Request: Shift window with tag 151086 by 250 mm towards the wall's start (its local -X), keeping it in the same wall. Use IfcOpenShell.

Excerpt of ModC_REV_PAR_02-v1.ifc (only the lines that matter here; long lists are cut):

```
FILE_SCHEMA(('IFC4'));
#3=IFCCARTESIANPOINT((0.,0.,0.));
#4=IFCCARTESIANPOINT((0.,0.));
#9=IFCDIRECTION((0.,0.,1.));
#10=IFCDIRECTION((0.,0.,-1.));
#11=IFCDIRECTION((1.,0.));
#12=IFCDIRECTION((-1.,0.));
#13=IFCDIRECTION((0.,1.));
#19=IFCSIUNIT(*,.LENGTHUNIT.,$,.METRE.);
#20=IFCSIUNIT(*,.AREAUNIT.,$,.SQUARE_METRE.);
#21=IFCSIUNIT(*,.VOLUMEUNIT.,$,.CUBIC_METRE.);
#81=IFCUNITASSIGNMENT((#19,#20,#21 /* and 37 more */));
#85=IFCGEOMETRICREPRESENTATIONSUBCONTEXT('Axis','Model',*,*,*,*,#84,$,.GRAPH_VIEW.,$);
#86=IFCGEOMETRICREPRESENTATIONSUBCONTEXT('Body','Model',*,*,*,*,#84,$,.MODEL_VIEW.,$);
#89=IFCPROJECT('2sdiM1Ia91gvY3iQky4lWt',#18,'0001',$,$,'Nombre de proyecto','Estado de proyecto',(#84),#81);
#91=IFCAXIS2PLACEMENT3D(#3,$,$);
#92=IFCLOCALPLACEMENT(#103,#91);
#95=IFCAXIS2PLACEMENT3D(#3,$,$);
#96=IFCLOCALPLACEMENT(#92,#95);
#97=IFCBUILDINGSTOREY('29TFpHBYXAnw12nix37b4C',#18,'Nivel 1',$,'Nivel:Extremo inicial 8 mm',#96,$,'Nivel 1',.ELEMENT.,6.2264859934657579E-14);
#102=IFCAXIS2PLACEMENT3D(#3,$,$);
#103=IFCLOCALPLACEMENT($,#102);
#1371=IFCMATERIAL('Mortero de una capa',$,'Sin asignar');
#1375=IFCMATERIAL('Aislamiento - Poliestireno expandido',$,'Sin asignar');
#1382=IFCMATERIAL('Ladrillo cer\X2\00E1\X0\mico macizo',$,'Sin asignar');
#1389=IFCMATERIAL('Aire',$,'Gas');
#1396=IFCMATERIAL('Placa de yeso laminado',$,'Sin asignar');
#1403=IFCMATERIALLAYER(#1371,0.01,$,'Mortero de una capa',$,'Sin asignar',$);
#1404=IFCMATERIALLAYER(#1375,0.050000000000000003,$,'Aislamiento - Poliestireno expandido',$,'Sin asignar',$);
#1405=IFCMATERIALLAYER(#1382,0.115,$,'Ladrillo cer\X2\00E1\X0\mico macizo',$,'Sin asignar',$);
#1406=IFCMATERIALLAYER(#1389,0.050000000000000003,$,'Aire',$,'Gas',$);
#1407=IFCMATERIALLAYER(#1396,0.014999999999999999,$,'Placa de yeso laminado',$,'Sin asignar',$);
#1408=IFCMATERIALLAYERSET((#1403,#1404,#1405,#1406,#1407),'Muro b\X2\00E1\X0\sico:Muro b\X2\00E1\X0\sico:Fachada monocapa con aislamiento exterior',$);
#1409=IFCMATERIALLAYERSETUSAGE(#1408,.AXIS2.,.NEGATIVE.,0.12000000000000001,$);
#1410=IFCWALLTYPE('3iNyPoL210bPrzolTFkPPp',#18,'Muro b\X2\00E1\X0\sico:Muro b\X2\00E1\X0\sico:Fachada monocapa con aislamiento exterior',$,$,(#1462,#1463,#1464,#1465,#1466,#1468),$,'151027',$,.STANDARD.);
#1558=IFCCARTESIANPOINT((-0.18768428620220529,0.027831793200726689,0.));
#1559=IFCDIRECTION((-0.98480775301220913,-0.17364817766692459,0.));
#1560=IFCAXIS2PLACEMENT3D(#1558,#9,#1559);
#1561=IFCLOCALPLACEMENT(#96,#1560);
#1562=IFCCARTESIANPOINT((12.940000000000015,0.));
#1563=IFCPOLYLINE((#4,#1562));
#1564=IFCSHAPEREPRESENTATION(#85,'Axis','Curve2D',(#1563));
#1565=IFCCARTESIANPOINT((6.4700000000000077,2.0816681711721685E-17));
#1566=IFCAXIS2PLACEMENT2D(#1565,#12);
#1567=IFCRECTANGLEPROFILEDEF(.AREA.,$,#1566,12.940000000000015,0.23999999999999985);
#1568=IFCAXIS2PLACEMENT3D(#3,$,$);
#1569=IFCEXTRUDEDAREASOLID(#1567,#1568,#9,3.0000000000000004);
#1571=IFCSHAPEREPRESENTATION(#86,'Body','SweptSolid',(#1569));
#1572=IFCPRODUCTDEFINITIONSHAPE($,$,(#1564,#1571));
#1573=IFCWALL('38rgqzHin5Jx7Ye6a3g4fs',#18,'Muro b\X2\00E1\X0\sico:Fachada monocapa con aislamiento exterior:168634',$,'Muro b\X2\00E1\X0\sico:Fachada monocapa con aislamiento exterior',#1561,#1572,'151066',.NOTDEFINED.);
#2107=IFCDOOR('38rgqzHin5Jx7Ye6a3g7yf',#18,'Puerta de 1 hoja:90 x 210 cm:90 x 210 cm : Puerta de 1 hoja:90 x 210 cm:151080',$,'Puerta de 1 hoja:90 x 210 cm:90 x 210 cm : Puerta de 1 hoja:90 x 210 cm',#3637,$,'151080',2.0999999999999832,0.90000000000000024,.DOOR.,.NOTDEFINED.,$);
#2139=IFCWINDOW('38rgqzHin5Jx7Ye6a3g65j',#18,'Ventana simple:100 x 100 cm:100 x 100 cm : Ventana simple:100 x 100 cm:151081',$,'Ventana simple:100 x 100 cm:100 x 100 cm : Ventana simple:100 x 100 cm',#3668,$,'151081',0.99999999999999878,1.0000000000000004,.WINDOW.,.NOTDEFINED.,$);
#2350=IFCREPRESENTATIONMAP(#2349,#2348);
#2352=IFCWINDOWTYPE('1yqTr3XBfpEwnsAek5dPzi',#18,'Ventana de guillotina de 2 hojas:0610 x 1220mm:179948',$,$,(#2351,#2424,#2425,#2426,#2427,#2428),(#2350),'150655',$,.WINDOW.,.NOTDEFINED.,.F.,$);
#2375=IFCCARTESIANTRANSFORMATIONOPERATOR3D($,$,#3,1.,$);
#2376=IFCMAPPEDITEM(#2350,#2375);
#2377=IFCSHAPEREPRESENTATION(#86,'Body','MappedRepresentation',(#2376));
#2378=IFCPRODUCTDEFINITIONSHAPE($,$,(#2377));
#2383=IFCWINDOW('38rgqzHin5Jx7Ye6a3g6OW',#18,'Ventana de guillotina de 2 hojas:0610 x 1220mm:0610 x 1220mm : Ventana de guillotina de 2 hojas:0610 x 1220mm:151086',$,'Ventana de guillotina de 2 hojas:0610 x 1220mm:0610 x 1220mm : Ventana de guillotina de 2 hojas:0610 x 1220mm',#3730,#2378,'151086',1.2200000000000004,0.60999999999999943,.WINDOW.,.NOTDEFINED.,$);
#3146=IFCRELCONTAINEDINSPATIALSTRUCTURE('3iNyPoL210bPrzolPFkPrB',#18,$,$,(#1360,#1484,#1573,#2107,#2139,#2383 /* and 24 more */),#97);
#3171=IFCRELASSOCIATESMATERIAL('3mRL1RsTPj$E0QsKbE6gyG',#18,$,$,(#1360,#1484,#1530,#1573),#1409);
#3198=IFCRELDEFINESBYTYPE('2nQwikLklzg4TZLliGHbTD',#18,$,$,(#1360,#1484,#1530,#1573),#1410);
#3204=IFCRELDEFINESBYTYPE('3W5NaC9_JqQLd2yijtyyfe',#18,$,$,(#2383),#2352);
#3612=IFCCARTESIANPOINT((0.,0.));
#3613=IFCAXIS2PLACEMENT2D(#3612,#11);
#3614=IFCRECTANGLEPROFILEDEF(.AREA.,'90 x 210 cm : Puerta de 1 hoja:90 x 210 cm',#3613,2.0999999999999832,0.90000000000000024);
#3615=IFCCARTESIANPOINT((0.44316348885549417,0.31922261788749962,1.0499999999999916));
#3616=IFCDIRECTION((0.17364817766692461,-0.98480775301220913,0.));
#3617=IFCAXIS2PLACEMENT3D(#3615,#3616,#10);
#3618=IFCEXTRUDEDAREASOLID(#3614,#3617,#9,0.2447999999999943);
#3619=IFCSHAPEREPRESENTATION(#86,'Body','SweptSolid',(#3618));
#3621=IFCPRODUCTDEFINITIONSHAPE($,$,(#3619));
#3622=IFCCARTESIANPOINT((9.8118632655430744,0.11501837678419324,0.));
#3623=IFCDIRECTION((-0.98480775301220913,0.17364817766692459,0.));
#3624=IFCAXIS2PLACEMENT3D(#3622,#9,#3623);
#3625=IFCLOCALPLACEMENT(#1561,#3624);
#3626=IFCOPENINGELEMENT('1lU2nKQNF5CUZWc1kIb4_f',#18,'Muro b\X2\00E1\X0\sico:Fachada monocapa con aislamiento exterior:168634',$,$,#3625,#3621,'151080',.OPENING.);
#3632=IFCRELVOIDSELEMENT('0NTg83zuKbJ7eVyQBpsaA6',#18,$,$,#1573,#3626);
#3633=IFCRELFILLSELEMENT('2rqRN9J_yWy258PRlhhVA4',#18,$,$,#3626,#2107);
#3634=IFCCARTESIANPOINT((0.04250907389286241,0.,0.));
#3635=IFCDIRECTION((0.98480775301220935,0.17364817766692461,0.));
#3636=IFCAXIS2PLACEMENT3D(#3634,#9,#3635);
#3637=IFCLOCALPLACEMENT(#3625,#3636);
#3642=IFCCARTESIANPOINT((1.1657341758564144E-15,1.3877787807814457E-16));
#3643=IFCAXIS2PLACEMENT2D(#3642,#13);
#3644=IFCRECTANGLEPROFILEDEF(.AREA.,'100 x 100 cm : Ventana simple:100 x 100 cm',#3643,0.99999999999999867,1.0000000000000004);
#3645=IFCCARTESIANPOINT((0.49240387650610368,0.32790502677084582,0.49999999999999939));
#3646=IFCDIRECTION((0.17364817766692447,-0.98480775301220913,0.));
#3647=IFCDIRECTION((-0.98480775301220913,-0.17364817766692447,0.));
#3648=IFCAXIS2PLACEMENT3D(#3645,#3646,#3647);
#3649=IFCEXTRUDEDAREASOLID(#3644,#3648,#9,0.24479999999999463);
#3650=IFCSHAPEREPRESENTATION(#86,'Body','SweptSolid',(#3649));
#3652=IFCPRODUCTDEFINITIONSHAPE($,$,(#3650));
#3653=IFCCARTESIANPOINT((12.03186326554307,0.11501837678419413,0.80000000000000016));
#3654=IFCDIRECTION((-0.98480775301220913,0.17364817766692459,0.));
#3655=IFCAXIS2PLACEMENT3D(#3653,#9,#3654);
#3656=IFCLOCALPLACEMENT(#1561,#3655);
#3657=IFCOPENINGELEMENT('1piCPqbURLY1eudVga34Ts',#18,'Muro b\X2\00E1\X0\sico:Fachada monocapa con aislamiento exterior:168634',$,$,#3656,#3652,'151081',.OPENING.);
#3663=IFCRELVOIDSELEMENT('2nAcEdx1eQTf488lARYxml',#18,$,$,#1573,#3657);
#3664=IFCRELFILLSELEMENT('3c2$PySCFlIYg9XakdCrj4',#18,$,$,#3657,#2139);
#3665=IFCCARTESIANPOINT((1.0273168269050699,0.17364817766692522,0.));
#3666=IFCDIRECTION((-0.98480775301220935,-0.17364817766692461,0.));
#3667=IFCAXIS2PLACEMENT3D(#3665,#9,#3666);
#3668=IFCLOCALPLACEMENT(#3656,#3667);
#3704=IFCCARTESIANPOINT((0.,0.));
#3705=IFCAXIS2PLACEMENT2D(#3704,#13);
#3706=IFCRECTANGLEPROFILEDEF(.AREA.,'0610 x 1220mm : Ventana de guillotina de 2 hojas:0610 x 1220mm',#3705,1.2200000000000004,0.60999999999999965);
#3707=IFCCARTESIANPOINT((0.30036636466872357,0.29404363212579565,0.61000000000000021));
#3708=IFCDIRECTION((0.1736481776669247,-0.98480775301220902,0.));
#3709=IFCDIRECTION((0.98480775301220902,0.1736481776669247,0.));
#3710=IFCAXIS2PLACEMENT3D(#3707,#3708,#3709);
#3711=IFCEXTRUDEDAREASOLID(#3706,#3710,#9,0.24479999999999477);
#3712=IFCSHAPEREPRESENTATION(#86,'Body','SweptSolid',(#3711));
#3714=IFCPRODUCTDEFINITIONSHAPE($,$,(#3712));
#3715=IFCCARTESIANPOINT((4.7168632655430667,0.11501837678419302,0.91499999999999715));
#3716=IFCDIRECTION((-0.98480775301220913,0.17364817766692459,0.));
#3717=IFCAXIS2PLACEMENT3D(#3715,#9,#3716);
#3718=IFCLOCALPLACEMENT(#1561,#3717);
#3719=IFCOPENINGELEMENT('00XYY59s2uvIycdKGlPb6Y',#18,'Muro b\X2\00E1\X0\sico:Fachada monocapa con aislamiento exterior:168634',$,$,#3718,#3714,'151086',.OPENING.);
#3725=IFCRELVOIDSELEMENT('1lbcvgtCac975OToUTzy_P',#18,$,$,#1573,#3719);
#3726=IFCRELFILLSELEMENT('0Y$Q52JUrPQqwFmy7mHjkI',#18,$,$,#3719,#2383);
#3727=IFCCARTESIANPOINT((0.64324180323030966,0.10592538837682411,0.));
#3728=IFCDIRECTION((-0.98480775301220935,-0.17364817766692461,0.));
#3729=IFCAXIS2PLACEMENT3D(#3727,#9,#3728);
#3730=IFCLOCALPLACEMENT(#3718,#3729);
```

```python
import ifcopenshell
import ifcopenshell.api.geometry
import ifcopenshell.util.placement
import ifcopenshell.util.unit

model = ifcopenshell.open("ModC_REV_PAR_02-v1.ifc")
unit_scale = ifcopenshell.util.unit.calculate_unit_scale(model)

window = model.by_guid("38rgqzHin5Jx7Ye6a3g6OW")
opening = window.FillsVoids[0].RelatingOpeningElement
wall = opening.VoidsElements[0].RelatingBuildingElement

wall_matrix = ifcopenshell.util.placement.get_local_placement(wall.ObjectPlacement)
shift = wall_matrix[:3, 0] * -0.25 / unit_scale
before = ifcopenshell.util.placement.get_local_placement(window.ObjectPlacement)[:3, 3].copy()

# The window is placed relative to its opening, so it follows when the opening moves.
matrix = ifcopenshell.util.placement.get_local_placement(opening.ObjectPlacement)
matrix[:3, 3] += shift
ifcopenshell.api.geometry.edit_object_placement(
    model, product=opening, matrix=matrix, is_si=False, should_transform_children=True
)

after = ifcopenshell.util.placement.get_local_placement(window.ObjectPlacement)[:3, 3]
print("window moved by", (after - before).round(3) + 0.0)

model.write("ModC_REV_PAR_02-v1_edited.ifc")
```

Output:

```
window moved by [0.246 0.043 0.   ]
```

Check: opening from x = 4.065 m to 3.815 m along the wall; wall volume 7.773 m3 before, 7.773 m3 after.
